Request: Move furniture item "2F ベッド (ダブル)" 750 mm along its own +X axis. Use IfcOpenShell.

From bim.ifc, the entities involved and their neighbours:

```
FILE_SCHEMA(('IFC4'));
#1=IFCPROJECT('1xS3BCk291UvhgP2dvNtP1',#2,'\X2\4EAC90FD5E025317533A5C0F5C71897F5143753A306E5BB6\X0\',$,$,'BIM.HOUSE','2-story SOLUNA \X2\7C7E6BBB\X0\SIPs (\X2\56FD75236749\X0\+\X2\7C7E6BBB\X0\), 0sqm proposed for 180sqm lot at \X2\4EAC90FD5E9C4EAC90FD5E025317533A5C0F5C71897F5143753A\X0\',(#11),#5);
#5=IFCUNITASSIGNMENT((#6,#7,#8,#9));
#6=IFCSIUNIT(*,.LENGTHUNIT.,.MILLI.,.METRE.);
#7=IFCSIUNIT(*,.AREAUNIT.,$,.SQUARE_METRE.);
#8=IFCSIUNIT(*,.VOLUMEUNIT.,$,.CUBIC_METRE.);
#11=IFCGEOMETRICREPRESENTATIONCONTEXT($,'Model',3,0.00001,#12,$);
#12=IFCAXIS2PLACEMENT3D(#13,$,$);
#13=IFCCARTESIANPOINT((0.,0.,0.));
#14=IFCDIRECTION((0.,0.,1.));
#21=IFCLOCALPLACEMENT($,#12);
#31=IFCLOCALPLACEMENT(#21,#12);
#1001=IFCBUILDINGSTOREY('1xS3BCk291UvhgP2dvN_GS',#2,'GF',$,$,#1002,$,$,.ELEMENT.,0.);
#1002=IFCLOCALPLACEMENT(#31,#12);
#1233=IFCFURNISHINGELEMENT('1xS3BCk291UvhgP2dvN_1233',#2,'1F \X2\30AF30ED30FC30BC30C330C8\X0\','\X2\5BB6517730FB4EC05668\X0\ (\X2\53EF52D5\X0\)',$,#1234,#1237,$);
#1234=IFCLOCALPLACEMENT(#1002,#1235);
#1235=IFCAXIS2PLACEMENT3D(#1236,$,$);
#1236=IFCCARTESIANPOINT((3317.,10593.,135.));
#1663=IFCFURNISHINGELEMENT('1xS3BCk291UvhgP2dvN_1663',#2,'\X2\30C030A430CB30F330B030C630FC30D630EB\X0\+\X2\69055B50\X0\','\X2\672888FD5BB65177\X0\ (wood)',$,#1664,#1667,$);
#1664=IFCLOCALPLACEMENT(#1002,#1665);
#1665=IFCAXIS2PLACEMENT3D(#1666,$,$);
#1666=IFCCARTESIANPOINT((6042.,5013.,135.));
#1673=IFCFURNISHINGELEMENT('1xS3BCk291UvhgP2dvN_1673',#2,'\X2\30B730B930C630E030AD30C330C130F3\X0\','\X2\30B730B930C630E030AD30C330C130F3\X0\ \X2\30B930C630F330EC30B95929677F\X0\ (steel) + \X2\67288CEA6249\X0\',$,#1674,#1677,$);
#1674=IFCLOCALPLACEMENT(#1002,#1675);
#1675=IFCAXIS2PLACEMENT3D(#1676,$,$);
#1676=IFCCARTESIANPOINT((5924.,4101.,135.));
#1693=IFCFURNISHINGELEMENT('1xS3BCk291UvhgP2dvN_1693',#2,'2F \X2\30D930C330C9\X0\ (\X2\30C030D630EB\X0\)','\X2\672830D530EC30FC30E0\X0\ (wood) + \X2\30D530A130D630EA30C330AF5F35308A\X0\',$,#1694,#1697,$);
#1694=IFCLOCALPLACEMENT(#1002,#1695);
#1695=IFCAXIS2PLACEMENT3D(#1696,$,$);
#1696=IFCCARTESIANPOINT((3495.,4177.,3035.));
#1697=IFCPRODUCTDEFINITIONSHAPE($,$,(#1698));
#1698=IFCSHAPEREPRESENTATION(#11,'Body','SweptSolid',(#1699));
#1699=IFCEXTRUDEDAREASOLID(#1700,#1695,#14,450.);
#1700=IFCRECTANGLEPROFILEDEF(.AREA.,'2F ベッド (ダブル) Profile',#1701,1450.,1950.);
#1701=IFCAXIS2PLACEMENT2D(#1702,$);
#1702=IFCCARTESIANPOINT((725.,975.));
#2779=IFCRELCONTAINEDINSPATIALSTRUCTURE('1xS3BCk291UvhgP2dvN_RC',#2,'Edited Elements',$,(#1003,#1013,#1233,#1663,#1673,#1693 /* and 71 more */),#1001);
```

```python
import ifcopenshell
import ifcopenshell.api.geometry
import ifcopenshell.util.placement
import ifcopenshell.util.unit

model = ifcopenshell.open("bim.ifc")
unit_scale = ifcopenshell.util.unit.calculate_unit_scale(model)

item = model.by_guid("1xS3BCk291UvhgP2dvN_1693")
matrix = ifcopenshell.util.placement.get_local_placement(item.ObjectPlacement)
matrix[:3, 3] += matrix[:3, 0] * 0.75 / unit_scale
ifcopenshell.api.geometry.edit_object_placement(model, product=item, matrix=matrix, is_si=False)

print(ifcopenshell.util.placement.get_local_placement(item.ObjectPlacement).round(3) + 0.0)

model.write("bim_v2.ifc")
```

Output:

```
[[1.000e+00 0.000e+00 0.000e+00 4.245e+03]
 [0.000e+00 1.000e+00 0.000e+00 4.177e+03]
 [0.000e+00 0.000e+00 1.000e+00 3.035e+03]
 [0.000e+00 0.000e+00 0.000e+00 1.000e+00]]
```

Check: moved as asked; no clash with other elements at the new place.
